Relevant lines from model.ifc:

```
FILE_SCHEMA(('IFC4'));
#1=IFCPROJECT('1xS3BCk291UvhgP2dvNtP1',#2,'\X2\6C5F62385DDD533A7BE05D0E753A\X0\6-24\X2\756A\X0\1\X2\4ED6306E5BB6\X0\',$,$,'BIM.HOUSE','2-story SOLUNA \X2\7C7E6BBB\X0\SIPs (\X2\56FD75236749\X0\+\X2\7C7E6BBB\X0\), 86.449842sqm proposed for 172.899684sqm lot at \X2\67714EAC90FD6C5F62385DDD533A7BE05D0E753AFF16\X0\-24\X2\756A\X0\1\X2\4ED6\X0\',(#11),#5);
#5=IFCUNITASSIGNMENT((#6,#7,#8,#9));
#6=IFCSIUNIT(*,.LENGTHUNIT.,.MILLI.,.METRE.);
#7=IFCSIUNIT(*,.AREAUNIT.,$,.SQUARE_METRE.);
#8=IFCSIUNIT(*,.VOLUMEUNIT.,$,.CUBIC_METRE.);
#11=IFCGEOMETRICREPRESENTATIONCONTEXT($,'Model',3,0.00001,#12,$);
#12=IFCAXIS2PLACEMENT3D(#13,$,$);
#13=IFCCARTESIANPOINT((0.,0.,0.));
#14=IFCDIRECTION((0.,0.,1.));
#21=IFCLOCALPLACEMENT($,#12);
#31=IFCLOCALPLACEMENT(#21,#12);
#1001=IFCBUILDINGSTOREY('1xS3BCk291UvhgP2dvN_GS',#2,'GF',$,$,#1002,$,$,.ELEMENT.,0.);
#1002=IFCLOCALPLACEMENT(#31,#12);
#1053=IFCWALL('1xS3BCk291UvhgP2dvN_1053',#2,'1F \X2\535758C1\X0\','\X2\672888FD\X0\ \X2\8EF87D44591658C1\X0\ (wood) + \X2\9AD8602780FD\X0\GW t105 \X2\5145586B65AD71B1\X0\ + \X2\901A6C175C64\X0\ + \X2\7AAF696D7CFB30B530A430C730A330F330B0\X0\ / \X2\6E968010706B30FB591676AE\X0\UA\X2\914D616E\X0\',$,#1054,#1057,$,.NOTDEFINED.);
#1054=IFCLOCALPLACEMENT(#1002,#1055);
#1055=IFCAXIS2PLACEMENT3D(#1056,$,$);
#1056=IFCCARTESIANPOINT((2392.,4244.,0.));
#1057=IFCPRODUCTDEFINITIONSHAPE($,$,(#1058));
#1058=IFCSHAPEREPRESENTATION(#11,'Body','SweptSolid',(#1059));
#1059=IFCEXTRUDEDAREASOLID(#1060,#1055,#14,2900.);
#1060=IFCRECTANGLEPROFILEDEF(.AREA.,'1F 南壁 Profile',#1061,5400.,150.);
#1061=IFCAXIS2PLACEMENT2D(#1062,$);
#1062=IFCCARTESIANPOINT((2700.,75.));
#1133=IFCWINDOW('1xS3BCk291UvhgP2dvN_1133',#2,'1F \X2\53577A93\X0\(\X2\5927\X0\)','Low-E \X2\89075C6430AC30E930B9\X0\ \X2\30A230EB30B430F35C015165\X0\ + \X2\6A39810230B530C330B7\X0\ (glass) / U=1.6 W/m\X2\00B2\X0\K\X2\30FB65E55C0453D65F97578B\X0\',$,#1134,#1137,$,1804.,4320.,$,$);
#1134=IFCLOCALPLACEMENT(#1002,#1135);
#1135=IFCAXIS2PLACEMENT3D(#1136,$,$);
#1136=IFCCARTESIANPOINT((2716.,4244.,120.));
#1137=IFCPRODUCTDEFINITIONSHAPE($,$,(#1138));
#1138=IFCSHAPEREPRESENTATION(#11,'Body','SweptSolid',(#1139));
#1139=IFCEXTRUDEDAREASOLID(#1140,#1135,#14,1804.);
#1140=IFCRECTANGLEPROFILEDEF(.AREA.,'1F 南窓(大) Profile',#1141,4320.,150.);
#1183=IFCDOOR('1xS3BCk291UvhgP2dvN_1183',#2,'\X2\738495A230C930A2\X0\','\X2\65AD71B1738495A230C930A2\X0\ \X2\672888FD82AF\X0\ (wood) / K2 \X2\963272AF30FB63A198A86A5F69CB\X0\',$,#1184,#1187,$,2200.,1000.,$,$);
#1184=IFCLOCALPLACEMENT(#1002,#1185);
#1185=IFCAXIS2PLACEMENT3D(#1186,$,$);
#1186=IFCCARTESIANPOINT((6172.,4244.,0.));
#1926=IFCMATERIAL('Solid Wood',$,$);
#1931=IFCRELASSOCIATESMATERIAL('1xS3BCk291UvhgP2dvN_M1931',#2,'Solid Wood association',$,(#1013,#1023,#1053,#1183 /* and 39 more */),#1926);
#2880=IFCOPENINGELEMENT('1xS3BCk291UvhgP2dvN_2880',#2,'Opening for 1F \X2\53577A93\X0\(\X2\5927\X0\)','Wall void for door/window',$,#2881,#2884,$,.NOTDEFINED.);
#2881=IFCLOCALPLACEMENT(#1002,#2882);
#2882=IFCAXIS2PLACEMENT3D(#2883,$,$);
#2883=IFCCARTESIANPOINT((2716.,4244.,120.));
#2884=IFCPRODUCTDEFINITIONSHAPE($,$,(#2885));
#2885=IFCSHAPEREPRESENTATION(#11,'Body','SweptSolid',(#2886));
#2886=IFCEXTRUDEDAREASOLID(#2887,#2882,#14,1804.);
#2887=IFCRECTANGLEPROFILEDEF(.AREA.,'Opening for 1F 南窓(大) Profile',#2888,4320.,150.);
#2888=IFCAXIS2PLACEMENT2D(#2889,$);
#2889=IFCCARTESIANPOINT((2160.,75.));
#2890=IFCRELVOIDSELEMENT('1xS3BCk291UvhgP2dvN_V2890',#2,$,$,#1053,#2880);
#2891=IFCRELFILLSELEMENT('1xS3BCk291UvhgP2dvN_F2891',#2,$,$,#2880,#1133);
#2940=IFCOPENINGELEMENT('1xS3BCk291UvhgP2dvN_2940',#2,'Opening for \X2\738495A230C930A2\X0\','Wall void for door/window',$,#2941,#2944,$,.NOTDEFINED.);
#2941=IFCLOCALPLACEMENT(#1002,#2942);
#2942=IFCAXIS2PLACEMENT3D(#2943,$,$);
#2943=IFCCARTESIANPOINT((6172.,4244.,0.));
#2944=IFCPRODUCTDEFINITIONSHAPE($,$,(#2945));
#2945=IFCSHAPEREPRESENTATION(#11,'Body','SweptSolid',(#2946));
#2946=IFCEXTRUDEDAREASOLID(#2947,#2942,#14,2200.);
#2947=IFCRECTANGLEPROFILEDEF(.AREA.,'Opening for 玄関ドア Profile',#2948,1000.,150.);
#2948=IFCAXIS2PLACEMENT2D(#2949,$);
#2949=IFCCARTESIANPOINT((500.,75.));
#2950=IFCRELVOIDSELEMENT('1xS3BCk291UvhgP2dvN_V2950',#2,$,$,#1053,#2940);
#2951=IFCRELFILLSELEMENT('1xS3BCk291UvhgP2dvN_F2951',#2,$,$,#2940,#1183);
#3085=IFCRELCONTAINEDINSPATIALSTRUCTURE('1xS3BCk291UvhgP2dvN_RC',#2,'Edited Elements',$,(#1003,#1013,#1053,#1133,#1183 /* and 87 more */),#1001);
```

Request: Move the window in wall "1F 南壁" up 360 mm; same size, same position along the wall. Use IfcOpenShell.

```python
import numpy as np
import ifcopenshell
import ifcopenshell.api.geometry
import ifcopenshell.util.placement
import ifcopenshell.util.unit

model = ifcopenshell.open("model.ifc")
unit_scale = ifcopenshell.util.unit.calculate_unit_scale(model)

window = model.by_guid("1xS3BCk291UvhgP2dvN_1133")
opening = window.FillsVoids[0].RelatingOpeningElement
dz = 360.0

shift = np.array([0.0, 0.0, dz])
# The window is not placed relative to its opening, so move both.
for product in (opening, window):
    matrix = ifcopenshell.util.placement.get_local_placement(product.ObjectPlacement)
    matrix[:3, 3] += shift
    ifcopenshell.api.geometry.edit_object_placement(model, product=product, matrix=matrix, is_si=False)

print(f"moved by {dz * unit_scale:+.3f} m")

model.write("model_updated.ifc")
```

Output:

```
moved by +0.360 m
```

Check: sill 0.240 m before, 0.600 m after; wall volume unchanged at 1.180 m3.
